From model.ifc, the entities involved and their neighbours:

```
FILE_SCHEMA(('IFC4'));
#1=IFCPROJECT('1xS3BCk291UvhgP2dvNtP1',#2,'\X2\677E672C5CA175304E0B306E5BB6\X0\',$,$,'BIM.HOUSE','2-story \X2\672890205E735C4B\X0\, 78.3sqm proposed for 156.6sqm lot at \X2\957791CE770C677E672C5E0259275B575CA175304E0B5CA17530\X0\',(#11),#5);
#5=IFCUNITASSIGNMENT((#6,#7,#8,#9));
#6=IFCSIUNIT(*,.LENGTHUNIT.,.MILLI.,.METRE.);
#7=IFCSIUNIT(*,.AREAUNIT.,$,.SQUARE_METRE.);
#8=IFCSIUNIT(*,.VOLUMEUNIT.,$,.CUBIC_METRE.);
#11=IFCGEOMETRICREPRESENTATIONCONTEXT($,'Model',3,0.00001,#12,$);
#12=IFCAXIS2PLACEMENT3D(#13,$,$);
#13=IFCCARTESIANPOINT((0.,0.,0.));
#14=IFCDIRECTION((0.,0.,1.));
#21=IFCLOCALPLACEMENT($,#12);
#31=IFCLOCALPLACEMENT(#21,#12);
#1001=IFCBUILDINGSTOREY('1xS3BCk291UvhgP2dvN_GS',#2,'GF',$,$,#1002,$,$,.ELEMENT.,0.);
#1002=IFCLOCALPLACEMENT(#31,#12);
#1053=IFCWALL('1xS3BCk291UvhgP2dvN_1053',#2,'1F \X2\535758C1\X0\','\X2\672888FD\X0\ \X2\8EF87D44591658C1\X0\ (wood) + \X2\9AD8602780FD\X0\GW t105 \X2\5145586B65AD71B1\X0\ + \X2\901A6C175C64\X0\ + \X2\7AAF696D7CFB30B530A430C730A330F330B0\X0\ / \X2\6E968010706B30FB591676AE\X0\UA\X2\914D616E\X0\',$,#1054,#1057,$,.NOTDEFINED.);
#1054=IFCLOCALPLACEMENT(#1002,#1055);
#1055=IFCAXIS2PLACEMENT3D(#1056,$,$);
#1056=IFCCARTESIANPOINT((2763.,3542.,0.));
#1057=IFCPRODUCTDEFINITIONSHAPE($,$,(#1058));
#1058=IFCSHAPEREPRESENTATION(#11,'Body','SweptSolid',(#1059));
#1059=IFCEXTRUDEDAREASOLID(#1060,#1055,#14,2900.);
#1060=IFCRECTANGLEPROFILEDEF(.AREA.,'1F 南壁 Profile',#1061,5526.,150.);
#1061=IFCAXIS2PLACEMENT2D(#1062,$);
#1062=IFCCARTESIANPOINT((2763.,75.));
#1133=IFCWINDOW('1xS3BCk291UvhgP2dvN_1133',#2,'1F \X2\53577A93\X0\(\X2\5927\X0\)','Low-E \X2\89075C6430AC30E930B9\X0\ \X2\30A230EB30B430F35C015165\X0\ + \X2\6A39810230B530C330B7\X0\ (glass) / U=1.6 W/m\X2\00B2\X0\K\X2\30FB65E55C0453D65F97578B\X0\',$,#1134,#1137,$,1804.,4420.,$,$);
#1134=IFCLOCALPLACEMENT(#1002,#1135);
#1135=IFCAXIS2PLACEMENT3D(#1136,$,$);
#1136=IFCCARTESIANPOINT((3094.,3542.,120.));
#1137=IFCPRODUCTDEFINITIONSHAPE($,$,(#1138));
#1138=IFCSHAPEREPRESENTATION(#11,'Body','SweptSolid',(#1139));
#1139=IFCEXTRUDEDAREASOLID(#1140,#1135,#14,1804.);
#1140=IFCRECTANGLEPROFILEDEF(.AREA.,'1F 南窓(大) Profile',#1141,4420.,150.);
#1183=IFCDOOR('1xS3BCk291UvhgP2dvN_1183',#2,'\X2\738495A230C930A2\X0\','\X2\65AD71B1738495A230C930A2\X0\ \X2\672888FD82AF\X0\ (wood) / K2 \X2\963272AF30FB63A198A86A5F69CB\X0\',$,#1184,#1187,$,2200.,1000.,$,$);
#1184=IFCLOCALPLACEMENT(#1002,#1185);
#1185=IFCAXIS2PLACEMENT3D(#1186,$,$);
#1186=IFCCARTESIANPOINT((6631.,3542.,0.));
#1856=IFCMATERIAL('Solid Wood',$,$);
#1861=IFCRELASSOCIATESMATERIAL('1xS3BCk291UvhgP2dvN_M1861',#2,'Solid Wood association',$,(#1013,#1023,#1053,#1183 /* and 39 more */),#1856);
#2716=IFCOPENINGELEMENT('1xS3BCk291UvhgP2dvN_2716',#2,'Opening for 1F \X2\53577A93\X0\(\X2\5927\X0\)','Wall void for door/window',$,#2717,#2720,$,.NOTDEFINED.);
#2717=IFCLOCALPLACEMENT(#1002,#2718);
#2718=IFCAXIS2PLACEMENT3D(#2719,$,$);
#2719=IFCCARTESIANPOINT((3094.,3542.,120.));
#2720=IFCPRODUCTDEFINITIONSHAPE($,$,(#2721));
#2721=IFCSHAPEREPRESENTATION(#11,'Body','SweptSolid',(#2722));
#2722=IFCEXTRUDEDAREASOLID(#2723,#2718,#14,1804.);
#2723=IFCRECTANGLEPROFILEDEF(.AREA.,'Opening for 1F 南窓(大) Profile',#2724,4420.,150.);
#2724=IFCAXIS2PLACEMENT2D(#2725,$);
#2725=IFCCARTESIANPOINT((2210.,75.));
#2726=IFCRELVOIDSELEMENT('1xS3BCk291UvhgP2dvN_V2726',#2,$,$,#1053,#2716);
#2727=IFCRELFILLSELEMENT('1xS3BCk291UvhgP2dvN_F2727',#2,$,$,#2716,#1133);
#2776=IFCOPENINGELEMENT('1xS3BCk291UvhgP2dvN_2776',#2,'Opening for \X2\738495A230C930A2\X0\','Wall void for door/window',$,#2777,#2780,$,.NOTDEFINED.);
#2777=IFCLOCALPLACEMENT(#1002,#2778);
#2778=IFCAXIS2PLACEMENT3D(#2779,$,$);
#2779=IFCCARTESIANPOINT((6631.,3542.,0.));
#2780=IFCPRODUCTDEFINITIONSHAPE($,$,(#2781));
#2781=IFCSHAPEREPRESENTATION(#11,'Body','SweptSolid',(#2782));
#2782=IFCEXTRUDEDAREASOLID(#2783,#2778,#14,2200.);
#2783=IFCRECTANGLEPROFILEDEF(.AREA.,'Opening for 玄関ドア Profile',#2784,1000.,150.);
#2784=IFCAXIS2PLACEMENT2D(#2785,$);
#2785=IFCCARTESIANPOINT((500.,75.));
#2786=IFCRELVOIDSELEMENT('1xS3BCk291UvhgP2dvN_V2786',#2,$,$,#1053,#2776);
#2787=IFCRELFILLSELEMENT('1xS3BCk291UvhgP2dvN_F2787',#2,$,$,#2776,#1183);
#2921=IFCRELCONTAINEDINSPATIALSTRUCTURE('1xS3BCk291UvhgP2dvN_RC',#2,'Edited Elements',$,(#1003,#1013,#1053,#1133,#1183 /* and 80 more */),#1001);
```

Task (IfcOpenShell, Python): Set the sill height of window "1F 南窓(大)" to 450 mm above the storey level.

```python
import numpy as np
import ifcopenshell
import ifcopenshell.api.geometry
import ifcopenshell.geom
import ifcopenshell.util.element
import ifcopenshell.util.placement
import ifcopenshell.util.shape
import ifcopenshell.util.unit

model = ifcopenshell.open("model.ifc")
unit_scale = ifcopenshell.util.unit.calculate_unit_scale(model)

window = model.by_id(1133)
opening = window.FillsVoids[0].RelatingOpeningElement
storey = ifcopenshell.util.element.get_container(window, ifc_class="IfcBuildingStorey")
level = ifcopenshell.util.placement.get_local_placement(storey.ObjectPlacement)[2, 3]

# The opening's origin need not be at the sill, so measure its lowest point.
shape = ifcopenshell.geom.create_shape(ifcopenshell.geom.settings(), opening)
bottom = ifcopenshell.util.shape.get_shape_bottom_elevation(shape, shape.geometry) / unit_scale
dz = level + 450.0 - bottom

shift = np.array([0.0, 0.0, dz])
# The window is not placed relative to its opening, so move both.
for product in (opening, window):
    matrix = ifcopenshell.util.placement.get_local_placement(product.ObjectPlacement)
    matrix[:3, 3] += shift
    ifcopenshell.api.geometry.edit_object_placement(model, product=product, matrix=matrix, is_si=False)

print(f"moved by {dz * unit_scale:+.3f} m")

model.write("model_edited.ifc")
```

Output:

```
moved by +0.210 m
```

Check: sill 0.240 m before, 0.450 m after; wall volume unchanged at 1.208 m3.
